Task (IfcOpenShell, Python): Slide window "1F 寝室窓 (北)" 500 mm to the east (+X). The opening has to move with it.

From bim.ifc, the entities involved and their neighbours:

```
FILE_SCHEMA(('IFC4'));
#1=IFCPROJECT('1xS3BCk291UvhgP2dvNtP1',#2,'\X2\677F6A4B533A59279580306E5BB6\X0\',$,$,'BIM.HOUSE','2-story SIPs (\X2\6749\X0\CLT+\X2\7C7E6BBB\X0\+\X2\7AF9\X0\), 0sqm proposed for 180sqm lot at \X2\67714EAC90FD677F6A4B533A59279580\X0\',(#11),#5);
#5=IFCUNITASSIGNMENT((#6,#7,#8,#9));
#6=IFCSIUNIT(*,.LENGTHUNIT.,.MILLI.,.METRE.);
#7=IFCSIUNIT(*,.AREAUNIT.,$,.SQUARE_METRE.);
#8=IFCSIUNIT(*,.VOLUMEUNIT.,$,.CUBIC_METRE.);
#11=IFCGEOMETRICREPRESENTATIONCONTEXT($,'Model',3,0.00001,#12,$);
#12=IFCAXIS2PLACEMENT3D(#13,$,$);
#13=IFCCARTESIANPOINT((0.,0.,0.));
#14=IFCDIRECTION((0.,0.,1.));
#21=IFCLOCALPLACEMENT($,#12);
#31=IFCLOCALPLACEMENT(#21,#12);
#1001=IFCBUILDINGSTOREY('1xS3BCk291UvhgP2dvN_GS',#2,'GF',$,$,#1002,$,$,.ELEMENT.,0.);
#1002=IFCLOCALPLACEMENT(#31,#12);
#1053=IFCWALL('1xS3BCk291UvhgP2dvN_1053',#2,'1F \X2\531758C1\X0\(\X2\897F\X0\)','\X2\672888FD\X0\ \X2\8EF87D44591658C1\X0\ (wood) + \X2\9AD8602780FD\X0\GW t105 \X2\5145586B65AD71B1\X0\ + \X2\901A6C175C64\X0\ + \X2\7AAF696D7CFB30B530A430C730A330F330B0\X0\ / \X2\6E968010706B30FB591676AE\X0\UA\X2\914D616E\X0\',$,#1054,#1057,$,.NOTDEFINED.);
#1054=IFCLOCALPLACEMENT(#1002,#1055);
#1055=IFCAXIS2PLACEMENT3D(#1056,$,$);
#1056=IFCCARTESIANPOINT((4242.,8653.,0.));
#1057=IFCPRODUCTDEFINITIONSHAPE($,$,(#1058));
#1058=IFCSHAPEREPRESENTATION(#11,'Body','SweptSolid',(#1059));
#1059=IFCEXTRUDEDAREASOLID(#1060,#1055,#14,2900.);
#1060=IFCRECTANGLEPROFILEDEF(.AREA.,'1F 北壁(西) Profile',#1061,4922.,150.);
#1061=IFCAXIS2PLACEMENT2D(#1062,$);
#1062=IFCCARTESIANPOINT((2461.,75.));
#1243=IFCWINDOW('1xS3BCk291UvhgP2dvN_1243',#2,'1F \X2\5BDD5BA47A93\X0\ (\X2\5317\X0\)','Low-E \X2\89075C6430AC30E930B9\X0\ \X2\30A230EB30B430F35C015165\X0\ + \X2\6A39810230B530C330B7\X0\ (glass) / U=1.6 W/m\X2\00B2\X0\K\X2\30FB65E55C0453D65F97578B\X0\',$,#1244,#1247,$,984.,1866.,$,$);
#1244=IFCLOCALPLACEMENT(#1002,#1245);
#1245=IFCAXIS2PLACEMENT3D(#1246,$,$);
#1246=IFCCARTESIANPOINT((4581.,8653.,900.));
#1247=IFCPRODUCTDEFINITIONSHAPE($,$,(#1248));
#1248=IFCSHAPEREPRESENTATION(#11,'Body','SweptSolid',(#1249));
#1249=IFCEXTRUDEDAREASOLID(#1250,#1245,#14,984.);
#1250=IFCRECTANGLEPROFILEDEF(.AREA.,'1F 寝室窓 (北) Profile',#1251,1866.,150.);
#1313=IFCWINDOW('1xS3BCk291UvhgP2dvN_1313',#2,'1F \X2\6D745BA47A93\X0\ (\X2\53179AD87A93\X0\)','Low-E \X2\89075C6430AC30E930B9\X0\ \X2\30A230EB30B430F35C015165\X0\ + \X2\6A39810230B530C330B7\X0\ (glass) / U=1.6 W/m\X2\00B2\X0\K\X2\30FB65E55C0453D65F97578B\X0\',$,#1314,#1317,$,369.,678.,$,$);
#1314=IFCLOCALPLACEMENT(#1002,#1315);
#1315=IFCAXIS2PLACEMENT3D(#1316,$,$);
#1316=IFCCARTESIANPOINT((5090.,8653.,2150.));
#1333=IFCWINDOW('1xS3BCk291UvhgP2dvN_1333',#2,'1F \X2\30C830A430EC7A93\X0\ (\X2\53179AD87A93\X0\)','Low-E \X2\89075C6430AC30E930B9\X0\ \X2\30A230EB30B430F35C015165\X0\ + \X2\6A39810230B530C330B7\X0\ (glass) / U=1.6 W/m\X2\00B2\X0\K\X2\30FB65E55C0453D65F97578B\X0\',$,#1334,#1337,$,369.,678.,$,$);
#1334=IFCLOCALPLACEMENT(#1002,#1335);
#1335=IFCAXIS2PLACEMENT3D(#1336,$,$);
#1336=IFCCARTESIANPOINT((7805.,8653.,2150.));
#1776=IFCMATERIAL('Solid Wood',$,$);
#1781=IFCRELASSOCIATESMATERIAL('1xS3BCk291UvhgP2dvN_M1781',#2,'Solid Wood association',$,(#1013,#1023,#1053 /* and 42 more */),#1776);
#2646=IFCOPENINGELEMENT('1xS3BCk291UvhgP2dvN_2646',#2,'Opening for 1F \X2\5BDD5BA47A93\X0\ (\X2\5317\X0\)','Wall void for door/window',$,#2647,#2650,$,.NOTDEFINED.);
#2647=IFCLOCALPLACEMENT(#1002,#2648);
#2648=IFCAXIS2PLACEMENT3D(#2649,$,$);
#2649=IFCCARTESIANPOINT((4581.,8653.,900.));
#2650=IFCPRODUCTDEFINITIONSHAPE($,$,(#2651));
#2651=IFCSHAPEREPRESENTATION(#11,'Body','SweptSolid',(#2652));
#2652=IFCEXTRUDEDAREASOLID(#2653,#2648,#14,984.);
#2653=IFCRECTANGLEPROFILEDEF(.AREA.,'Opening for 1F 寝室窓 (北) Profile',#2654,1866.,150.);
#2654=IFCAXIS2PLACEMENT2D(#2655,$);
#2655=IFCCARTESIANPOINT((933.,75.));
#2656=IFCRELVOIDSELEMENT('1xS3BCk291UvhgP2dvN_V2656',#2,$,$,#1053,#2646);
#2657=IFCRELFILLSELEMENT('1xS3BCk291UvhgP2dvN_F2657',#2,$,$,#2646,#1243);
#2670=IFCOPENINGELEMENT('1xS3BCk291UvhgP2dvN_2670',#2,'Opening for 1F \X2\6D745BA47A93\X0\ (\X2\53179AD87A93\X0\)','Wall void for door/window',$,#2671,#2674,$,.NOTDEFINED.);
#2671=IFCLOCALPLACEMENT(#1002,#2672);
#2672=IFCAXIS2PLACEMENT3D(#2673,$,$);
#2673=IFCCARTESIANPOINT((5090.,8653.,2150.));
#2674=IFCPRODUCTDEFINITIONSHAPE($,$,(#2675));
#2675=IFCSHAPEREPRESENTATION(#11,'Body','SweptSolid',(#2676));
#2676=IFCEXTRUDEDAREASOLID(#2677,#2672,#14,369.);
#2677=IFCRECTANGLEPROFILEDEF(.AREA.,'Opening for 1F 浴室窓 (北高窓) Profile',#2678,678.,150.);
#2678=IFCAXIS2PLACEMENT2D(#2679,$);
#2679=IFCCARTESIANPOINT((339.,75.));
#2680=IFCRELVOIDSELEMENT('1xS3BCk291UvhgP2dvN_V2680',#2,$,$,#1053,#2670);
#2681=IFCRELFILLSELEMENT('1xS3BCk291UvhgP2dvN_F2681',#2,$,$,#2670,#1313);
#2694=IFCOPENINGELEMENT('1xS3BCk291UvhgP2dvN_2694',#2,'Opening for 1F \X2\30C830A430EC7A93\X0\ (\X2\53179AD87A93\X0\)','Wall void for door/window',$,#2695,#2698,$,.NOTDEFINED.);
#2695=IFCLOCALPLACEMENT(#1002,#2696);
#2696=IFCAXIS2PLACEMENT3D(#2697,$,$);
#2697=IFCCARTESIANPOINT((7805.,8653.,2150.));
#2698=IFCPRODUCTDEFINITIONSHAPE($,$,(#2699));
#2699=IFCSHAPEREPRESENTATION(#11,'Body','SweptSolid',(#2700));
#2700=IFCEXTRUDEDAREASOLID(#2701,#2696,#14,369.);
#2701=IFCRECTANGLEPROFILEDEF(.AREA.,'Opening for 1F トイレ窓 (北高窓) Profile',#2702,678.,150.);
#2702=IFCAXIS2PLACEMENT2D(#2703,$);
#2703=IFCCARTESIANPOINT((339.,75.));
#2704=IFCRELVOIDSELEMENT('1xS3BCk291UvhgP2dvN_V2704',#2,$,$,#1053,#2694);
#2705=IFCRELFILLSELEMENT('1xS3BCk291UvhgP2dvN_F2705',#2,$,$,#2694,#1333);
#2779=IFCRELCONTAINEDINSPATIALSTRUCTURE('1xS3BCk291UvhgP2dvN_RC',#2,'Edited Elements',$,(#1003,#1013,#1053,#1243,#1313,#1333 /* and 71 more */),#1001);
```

```python
import ifcopenshell
import ifcopenshell.api.geometry
import ifcopenshell.util.placement
import ifcopenshell.util.unit

model = ifcopenshell.open("bim.ifc")
unit_scale = ifcopenshell.util.unit.calculate_unit_scale(model)

window = model.by_guid("1xS3BCk291UvhgP2dvN_1243")
opening = window.FillsVoids[0].RelatingOpeningElement
wall = opening.VoidsElements[0].RelatingBuildingElement

wall_matrix = ifcopenshell.util.placement.get_local_placement(wall.ObjectPlacement)
shift = wall_matrix[:3, 0] * 0.5 / unit_scale
before = ifcopenshell.util.placement.get_local_placement(window.ObjectPlacement)[:3, 3].copy()

# The window is not placed relative to its opening, so move both.
for product in (opening, window):
    matrix = ifcopenshell.util.placement.get_local_placement(product.ObjectPlacement)
    matrix[:3, 3] += shift
    ifcopenshell.api.geometry.edit_object_placement(model, product=product, matrix=matrix, is_si=False)

after = ifcopenshell.util.placement.get_local_placement(window.ObjectPlacement)[:3, 3]
print("window moved by", (after - before).round(3) + 0.0)

model.write("bim_v2.ifc")
```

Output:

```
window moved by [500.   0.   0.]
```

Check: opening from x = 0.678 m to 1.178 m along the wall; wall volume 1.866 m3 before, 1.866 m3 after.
